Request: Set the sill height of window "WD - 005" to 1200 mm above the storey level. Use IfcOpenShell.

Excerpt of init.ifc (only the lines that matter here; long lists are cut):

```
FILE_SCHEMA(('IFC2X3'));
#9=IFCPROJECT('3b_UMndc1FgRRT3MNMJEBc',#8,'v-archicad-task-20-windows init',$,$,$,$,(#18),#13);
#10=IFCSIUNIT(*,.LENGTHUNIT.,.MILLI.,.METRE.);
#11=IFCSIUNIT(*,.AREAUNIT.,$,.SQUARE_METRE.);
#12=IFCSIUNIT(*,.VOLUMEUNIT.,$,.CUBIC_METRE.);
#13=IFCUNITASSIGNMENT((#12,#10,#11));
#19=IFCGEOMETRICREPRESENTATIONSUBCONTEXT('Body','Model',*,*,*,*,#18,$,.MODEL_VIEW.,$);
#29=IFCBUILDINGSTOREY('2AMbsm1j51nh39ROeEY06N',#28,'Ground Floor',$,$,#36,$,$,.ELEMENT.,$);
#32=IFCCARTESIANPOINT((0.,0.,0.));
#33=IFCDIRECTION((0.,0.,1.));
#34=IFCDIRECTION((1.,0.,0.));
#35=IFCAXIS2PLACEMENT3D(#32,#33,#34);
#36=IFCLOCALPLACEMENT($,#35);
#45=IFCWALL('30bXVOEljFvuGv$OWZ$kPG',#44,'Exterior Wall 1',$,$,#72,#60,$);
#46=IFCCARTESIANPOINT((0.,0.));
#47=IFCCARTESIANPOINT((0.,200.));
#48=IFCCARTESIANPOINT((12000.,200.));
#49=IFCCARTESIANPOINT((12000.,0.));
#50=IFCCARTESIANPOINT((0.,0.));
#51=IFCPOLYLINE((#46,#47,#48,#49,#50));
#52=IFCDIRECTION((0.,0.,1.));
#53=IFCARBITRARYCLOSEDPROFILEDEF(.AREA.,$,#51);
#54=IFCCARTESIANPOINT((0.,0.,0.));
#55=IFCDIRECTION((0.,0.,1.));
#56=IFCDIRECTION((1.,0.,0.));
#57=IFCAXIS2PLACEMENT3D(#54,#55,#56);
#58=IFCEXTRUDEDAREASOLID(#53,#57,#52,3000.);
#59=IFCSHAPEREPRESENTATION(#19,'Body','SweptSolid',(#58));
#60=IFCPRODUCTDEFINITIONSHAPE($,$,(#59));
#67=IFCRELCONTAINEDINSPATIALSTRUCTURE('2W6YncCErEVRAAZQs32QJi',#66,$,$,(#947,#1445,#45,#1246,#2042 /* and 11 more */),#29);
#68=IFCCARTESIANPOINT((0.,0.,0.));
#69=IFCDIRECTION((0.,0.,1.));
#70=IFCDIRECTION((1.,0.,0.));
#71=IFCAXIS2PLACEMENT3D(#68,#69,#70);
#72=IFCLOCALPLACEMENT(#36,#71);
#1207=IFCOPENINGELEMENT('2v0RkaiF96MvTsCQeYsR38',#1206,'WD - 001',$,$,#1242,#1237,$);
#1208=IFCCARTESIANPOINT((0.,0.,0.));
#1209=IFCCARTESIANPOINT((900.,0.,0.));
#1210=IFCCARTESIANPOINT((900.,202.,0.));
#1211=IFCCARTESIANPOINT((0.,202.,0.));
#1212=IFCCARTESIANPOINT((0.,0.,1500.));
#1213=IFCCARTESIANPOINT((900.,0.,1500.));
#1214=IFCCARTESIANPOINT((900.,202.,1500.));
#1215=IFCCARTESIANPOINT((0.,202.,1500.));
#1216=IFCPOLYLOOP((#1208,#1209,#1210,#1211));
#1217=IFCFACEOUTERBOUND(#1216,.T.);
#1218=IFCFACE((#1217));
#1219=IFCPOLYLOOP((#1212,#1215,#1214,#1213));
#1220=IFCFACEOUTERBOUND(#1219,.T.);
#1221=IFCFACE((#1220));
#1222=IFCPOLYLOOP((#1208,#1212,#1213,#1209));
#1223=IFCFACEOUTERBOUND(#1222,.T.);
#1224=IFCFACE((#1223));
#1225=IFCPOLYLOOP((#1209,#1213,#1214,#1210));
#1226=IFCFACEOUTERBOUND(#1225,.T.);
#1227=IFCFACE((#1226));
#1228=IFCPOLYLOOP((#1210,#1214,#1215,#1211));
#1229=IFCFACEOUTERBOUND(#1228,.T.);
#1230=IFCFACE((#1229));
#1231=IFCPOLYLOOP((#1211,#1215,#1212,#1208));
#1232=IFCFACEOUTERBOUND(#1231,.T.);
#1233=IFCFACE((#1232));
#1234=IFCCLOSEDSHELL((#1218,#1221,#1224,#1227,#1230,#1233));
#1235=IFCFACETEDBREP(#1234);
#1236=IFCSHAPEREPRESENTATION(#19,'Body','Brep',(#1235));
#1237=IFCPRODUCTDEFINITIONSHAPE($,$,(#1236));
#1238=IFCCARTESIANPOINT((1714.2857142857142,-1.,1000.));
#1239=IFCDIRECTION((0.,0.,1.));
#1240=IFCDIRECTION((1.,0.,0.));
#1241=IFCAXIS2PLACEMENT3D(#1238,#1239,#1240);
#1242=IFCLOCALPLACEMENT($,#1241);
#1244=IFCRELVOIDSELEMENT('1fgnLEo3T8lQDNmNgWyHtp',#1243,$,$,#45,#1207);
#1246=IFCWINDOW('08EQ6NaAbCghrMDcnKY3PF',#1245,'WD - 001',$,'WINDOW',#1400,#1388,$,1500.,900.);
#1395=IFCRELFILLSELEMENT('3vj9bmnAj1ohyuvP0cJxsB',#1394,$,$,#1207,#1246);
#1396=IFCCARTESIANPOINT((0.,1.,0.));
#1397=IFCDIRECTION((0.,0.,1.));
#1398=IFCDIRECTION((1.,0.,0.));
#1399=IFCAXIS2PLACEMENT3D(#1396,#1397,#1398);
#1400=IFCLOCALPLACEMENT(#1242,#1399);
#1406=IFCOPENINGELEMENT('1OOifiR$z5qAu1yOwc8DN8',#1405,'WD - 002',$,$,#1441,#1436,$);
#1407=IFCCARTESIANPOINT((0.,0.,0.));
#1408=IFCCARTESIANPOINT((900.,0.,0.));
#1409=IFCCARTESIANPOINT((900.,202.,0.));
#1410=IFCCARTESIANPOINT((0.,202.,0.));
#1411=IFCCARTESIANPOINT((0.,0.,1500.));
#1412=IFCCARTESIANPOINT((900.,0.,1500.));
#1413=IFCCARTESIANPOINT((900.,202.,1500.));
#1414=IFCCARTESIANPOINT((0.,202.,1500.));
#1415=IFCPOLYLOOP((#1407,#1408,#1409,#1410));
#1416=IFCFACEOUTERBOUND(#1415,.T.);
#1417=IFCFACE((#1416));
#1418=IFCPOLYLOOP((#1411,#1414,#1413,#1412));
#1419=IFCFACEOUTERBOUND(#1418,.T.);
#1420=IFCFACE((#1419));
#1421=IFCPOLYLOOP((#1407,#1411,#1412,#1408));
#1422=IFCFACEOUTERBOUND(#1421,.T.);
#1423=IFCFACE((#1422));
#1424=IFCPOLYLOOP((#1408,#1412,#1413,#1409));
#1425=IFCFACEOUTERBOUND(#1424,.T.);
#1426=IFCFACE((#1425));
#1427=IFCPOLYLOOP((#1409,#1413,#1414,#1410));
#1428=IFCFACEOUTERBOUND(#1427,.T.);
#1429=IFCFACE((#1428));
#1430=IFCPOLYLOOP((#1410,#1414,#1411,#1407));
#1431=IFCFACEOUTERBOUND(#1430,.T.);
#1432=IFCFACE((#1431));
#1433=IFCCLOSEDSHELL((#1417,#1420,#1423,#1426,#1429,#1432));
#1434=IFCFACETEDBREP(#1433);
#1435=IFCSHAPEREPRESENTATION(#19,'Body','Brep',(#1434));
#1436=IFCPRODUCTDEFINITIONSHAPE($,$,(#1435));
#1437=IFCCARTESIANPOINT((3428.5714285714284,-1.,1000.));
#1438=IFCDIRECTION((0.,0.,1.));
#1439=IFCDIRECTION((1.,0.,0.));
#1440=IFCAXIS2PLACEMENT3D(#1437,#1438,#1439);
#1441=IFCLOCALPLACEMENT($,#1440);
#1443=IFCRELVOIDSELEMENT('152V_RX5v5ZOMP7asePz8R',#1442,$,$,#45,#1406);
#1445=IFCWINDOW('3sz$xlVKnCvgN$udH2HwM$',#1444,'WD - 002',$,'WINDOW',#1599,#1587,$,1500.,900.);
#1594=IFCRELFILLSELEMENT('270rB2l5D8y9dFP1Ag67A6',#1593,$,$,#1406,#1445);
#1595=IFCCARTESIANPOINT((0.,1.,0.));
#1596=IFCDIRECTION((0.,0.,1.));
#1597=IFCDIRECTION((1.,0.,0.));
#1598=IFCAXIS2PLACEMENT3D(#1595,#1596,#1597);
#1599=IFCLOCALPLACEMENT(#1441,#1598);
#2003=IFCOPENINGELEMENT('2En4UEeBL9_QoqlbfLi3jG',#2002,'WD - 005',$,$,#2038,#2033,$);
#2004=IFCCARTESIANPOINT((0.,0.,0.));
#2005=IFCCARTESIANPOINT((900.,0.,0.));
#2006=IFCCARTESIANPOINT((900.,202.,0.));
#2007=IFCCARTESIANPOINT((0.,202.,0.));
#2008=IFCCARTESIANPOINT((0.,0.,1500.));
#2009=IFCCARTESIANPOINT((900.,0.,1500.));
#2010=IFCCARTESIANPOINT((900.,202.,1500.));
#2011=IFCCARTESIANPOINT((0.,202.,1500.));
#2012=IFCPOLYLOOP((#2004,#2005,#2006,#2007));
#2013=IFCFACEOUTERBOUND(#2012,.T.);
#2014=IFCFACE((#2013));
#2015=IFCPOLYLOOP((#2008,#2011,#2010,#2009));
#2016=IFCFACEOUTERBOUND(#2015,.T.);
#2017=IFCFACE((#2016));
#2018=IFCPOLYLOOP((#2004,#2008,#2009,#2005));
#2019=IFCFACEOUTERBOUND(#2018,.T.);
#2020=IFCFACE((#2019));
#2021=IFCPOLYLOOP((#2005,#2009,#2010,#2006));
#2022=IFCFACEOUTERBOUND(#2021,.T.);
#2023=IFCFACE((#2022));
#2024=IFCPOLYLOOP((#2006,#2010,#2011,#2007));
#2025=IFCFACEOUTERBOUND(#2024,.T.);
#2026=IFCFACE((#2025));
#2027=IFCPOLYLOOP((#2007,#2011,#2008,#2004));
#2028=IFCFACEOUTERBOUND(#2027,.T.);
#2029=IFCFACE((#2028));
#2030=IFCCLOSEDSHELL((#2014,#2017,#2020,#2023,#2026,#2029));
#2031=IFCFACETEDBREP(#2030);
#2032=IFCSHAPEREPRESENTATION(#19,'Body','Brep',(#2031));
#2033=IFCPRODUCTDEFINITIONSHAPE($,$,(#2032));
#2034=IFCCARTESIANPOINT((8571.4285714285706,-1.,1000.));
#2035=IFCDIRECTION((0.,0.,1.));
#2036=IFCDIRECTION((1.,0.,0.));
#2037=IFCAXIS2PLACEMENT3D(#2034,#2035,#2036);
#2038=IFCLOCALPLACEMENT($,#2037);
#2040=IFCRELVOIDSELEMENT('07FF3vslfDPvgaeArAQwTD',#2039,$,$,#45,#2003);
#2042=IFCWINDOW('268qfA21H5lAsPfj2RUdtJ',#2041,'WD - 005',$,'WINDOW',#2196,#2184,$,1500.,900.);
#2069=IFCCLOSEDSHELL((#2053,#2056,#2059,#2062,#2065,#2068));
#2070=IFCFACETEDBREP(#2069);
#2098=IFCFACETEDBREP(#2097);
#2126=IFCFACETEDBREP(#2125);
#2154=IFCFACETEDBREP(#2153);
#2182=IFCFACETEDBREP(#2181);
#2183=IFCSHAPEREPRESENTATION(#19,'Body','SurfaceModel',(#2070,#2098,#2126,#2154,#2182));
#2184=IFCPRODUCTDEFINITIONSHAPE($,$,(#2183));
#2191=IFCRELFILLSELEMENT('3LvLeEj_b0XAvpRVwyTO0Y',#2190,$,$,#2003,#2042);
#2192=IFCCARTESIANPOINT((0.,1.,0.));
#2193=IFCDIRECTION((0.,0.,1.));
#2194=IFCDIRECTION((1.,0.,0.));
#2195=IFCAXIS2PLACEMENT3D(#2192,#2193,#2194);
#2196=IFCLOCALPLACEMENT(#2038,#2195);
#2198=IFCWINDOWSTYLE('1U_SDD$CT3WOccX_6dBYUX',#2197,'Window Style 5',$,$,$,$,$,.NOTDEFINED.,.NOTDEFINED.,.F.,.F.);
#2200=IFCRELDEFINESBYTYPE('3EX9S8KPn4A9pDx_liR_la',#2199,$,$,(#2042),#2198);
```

```python
import numpy as np
import ifcopenshell
import ifcopenshell.api.geometry
import ifcopenshell.geom
import ifcopenshell.util.element
import ifcopenshell.util.placement
import ifcopenshell.util.shape
import ifcopenshell.util.unit

model = ifcopenshell.open("init.ifc")
unit_scale = ifcopenshell.util.unit.calculate_unit_scale(model)

window = model.by_guid("268qfA21H5lAsPfj2RUdtJ")
opening = window.FillsVoids[0].RelatingOpeningElement
storey = ifcopenshell.util.element.get_container(window, ifc_class="IfcBuildingStorey")
level = ifcopenshell.util.placement.get_local_placement(storey.ObjectPlacement)[2, 3]

# The opening's origin need not be at the sill, so measure its lowest point.
shape = ifcopenshell.geom.create_shape(ifcopenshell.geom.settings(), opening)
bottom = ifcopenshell.util.shape.get_shape_bottom_elevation(shape, shape.geometry) / unit_scale
dz = level + 1200.0 - bottom

shift = np.array([0.0, 0.0, dz])
# The window is placed relative to its opening, so it follows when the opening moves.
matrix = ifcopenshell.util.placement.get_local_placement(opening.ObjectPlacement)
matrix[:3, 3] += shift
ifcopenshell.api.geometry.edit_object_placement(
    model, product=opening, matrix=matrix, is_si=False, should_transform_children=True
)

print(f"moved by {dz * unit_scale:+.3f} m")

model.write("init_rev.ifc")
```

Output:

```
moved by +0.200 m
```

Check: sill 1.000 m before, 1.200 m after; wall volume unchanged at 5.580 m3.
